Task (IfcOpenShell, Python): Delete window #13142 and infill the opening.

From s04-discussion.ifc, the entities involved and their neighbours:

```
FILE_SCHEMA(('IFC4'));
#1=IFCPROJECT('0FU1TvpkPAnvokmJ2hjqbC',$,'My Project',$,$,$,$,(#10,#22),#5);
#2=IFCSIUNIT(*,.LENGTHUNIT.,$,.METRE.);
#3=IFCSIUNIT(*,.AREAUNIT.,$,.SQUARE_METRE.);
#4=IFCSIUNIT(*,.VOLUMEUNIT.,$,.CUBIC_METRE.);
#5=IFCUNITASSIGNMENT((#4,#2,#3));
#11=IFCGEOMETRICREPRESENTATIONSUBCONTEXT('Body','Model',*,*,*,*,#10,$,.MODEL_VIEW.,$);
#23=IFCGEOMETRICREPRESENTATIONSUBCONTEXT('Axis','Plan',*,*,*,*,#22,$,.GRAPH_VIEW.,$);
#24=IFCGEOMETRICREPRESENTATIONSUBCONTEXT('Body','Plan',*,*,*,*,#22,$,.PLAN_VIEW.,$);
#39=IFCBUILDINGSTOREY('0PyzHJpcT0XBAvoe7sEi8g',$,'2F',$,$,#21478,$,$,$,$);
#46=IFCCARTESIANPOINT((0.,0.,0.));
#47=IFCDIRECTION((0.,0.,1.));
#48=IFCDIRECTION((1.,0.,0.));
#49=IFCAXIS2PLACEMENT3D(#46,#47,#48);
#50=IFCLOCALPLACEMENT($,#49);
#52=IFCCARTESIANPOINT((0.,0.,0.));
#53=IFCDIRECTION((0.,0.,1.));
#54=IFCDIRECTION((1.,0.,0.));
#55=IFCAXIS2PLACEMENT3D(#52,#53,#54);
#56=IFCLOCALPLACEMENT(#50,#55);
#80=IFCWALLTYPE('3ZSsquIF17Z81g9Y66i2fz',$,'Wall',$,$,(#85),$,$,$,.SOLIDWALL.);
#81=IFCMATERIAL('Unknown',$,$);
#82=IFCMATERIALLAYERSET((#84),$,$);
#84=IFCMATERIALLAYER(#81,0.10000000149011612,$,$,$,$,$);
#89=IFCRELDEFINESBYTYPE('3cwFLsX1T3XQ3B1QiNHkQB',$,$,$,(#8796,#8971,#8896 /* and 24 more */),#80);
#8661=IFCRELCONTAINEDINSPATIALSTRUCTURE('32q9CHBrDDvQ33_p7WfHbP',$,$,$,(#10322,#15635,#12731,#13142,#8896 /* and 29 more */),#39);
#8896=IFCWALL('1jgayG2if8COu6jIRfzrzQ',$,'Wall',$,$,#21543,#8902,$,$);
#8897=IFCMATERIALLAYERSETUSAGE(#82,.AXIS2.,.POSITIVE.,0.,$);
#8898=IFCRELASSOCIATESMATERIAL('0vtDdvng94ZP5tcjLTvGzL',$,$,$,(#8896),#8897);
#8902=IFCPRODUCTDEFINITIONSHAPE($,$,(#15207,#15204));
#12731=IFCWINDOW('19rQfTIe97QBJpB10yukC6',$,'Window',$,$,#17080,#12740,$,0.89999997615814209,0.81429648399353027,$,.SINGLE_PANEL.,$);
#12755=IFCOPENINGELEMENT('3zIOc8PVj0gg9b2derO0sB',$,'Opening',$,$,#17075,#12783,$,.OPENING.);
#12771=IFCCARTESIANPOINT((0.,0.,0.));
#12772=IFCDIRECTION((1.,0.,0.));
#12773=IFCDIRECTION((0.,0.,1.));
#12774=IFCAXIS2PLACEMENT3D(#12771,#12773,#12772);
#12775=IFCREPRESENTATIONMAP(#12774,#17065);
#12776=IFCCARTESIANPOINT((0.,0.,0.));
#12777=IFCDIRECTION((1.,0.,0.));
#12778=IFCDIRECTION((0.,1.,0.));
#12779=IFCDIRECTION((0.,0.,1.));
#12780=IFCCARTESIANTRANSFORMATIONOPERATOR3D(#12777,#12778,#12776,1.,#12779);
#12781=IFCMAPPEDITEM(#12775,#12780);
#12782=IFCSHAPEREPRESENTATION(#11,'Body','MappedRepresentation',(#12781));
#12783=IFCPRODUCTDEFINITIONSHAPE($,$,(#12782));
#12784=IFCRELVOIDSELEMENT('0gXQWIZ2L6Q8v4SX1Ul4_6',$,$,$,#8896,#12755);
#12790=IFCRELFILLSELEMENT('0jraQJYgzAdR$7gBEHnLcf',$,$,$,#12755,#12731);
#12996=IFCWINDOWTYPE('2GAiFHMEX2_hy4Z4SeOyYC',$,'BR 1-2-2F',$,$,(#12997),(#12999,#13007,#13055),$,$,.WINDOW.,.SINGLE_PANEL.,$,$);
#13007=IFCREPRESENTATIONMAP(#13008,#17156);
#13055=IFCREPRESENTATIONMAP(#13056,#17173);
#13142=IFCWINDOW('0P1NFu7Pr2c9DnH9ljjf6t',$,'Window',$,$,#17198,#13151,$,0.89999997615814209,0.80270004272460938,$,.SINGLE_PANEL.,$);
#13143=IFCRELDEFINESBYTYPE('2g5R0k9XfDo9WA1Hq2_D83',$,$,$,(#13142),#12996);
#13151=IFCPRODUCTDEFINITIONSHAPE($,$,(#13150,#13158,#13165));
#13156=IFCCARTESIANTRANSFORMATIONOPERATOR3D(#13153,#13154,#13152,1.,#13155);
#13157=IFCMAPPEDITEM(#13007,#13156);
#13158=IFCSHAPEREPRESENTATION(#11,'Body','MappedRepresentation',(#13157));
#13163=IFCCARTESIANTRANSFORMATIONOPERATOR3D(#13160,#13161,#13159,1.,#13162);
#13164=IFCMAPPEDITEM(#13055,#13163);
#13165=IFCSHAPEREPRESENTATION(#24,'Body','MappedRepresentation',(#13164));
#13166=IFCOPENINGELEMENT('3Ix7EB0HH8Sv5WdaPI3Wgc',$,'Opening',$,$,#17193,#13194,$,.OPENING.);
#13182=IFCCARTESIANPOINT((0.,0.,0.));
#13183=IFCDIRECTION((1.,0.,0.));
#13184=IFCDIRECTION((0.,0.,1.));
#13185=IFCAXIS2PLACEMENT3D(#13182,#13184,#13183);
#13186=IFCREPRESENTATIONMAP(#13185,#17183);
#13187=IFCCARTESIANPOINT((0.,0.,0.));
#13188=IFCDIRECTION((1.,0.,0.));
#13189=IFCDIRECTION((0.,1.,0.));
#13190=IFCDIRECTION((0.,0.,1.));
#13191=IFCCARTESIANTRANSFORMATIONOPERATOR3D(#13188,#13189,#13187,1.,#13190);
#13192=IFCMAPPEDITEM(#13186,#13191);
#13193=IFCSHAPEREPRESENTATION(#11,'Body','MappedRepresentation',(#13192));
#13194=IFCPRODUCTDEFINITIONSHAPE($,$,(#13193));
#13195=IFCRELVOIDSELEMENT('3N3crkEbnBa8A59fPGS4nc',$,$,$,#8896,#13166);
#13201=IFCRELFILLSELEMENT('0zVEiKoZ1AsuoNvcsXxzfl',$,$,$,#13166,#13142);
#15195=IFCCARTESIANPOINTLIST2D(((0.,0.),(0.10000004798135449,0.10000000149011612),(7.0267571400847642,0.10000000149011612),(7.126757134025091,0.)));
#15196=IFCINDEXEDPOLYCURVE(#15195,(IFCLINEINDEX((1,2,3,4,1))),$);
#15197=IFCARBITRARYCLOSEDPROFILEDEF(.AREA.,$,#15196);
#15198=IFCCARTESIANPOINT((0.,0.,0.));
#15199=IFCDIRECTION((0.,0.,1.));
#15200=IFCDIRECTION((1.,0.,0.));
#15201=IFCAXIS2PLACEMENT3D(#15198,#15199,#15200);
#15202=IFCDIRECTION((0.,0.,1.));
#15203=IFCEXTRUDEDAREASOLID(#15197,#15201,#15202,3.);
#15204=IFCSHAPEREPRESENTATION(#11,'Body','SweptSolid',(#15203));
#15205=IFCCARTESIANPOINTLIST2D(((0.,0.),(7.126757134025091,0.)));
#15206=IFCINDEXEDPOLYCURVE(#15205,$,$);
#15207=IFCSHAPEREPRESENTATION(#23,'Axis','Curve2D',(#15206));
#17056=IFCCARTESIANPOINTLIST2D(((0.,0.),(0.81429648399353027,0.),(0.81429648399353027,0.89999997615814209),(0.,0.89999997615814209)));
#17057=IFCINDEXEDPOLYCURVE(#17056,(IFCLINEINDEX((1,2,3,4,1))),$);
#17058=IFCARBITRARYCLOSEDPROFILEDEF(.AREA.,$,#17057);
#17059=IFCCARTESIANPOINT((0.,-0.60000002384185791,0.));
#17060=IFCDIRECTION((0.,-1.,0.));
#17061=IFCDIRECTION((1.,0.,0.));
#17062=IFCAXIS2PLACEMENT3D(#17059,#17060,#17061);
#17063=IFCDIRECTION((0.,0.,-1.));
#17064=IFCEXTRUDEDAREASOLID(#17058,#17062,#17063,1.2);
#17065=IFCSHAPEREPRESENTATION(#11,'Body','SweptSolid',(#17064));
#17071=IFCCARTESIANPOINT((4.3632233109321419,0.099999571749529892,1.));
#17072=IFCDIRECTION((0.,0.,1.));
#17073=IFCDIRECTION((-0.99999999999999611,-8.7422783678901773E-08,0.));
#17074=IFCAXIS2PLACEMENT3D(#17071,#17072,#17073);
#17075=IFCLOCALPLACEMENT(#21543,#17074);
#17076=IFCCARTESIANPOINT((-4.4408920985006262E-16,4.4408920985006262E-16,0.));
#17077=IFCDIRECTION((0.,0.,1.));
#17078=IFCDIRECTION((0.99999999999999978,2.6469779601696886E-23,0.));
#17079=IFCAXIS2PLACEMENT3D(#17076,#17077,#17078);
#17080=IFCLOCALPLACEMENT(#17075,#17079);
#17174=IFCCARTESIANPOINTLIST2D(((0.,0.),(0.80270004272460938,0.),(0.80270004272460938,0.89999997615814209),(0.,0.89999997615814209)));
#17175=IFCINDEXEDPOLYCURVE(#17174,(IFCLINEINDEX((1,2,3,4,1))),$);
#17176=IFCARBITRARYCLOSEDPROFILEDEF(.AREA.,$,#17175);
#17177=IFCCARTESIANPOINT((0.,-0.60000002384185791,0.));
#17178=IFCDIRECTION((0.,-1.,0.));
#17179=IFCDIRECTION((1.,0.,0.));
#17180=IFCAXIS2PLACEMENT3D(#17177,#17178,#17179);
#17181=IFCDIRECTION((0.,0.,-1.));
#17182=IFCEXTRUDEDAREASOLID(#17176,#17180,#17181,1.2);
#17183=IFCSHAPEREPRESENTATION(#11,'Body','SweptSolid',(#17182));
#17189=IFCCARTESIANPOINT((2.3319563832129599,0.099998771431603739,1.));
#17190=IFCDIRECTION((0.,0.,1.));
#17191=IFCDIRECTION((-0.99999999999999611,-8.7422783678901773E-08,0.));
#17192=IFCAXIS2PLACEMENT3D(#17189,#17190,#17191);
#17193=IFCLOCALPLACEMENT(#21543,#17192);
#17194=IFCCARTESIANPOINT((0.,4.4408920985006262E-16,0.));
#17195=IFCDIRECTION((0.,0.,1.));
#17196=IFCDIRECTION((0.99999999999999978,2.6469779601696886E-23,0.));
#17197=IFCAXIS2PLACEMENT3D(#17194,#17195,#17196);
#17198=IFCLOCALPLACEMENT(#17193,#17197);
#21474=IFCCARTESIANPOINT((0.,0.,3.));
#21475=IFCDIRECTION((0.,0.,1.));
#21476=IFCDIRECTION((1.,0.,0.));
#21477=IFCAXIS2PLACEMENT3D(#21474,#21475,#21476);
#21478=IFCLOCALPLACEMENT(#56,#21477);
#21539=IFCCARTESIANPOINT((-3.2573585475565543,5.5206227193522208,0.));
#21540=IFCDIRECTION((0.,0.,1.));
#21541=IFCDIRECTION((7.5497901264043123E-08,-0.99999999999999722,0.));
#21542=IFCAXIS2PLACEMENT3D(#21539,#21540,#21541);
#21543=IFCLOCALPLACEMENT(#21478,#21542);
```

```python
import ifcopenshell
import ifcopenshell.api.feature
import ifcopenshell.api.root
import ifcopenshell.geom
import ifcopenshell.util.shape

model = ifcopenshell.open("s04-discussion.ifc")
settings = ifcopenshell.geom.settings()


def volume(element):
    """Net volume in cubic metres, openings subtracted."""
    shape = ifcopenshell.geom.create_shape(settings, element)
    return ifcopenshell.util.shape.get_volume(shape.geometry)


window = model.by_id(13142)
opening = window.FillsVoids[0].RelatingOpeningElement
wall = opening.VoidsElements[0].RelatingBuildingElement
before = volume(wall)

ifcopenshell.api.root.remove_product(model, product=window)
ifcopenshell.api.feature.remove_feature(model, feature=opening)

after = volume(wall)

print(f"wall volume {before:.3f} -> {after:.3f} m3")

model.write("s04-discussion_v2.ifc")
```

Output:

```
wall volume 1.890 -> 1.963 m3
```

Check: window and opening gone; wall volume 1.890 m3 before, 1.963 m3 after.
